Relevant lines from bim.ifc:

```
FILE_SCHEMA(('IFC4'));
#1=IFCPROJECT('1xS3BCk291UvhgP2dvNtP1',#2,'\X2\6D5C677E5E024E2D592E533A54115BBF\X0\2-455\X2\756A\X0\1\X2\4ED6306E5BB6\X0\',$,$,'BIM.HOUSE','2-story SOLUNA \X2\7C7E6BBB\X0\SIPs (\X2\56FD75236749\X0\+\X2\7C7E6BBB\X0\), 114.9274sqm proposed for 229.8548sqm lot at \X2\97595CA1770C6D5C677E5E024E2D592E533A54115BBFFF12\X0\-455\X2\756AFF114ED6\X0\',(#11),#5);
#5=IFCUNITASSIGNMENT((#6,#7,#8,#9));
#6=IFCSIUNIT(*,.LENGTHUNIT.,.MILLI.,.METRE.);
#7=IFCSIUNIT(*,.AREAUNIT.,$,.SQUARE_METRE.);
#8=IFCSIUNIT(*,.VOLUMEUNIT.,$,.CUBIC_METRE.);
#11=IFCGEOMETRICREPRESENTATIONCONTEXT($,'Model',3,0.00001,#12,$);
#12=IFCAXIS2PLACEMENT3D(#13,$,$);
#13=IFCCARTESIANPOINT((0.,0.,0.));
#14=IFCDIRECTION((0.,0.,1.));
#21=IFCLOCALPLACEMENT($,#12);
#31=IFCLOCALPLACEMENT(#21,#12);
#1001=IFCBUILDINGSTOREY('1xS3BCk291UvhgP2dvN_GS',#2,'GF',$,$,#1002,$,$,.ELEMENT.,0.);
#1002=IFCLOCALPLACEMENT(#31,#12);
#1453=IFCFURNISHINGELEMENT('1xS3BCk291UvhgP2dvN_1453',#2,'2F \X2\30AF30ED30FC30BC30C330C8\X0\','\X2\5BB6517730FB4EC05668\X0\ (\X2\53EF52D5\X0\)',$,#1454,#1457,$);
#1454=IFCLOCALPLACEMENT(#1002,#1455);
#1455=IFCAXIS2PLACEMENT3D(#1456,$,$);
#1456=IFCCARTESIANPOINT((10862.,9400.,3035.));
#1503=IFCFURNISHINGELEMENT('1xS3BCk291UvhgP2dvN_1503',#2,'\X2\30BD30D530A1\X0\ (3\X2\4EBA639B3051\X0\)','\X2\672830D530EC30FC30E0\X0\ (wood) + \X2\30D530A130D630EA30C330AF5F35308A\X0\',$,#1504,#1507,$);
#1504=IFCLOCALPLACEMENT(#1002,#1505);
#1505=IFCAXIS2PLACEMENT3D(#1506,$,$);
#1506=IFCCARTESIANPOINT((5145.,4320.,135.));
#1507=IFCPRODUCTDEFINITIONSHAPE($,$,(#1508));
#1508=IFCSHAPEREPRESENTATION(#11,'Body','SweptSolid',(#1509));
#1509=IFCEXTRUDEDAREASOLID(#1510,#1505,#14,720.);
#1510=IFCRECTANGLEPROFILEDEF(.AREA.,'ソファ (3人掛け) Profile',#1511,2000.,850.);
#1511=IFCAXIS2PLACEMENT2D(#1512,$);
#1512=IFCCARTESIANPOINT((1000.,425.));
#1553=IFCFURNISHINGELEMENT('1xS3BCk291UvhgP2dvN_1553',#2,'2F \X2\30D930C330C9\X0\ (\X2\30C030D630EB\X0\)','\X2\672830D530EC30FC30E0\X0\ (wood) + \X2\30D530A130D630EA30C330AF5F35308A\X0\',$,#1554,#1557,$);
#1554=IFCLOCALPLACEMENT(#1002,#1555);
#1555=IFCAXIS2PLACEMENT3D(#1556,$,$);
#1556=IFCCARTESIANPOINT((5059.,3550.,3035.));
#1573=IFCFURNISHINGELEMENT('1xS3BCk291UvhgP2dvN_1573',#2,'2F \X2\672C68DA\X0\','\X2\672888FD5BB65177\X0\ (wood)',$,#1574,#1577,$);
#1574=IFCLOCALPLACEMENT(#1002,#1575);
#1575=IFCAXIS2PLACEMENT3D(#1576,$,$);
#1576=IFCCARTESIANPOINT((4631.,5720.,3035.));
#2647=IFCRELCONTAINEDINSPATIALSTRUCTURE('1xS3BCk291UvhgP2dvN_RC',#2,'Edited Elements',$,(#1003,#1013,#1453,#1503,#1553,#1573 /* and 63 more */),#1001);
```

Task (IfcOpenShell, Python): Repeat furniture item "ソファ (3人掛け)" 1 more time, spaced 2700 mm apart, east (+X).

```python
import numpy as np
import ifcopenshell
import ifcopenshell.api.geometry
import ifcopenshell.api.root
import ifcopenshell.util.element
import ifcopenshell.util.placement
import ifcopenshell.util.unit

model = ifcopenshell.open("bim.ifc")
unit_scale = ifcopenshell.util.unit.calculate_unit_scale(model)


def reuse_history(source, copy):
    """copy_class also copies each property set's owner history, people and application; keep the originals."""
    for rel in copy.IsDefinedBy:
        if rel.is_a("IfcRelDefinesByProperties") and (history := rel.RelatingPropertyDefinition.OwnerHistory):
            rel.RelatingPropertyDefinition.OwnerHistory = source.OwnerHistory
            ifcopenshell.util.element.remove_deep2(model, history)


source = model.by_guid("1xS3BCk291UvhgP2dvN_1503")
base = ifcopenshell.util.placement.get_local_placement(source.ObjectPlacement)
step = np.array([1.0, 0.0, 0.0]) * 2.7 / unit_scale

for i in range(1, 2):
    copy = ifcopenshell.api.root.copy_class(model, product=source)
    copy.Representation = ifcopenshell.util.element.copy_deep(
        model, source.Representation, exclude=["IfcGeometricRepresentationContext", "IfcRepresentationMap"]
    )
    reuse_history(source, copy)
    matrix = base.copy()
    matrix[:3, 3] += i * step
    print("added at", matrix[:3, 3].round(3) + 0.0)
    ifcopenshell.api.geometry.edit_object_placement(model, product=copy, matrix=matrix, is_si=False)

model.write("bim_rev.ifc")
```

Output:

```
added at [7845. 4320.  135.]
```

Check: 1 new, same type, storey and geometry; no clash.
